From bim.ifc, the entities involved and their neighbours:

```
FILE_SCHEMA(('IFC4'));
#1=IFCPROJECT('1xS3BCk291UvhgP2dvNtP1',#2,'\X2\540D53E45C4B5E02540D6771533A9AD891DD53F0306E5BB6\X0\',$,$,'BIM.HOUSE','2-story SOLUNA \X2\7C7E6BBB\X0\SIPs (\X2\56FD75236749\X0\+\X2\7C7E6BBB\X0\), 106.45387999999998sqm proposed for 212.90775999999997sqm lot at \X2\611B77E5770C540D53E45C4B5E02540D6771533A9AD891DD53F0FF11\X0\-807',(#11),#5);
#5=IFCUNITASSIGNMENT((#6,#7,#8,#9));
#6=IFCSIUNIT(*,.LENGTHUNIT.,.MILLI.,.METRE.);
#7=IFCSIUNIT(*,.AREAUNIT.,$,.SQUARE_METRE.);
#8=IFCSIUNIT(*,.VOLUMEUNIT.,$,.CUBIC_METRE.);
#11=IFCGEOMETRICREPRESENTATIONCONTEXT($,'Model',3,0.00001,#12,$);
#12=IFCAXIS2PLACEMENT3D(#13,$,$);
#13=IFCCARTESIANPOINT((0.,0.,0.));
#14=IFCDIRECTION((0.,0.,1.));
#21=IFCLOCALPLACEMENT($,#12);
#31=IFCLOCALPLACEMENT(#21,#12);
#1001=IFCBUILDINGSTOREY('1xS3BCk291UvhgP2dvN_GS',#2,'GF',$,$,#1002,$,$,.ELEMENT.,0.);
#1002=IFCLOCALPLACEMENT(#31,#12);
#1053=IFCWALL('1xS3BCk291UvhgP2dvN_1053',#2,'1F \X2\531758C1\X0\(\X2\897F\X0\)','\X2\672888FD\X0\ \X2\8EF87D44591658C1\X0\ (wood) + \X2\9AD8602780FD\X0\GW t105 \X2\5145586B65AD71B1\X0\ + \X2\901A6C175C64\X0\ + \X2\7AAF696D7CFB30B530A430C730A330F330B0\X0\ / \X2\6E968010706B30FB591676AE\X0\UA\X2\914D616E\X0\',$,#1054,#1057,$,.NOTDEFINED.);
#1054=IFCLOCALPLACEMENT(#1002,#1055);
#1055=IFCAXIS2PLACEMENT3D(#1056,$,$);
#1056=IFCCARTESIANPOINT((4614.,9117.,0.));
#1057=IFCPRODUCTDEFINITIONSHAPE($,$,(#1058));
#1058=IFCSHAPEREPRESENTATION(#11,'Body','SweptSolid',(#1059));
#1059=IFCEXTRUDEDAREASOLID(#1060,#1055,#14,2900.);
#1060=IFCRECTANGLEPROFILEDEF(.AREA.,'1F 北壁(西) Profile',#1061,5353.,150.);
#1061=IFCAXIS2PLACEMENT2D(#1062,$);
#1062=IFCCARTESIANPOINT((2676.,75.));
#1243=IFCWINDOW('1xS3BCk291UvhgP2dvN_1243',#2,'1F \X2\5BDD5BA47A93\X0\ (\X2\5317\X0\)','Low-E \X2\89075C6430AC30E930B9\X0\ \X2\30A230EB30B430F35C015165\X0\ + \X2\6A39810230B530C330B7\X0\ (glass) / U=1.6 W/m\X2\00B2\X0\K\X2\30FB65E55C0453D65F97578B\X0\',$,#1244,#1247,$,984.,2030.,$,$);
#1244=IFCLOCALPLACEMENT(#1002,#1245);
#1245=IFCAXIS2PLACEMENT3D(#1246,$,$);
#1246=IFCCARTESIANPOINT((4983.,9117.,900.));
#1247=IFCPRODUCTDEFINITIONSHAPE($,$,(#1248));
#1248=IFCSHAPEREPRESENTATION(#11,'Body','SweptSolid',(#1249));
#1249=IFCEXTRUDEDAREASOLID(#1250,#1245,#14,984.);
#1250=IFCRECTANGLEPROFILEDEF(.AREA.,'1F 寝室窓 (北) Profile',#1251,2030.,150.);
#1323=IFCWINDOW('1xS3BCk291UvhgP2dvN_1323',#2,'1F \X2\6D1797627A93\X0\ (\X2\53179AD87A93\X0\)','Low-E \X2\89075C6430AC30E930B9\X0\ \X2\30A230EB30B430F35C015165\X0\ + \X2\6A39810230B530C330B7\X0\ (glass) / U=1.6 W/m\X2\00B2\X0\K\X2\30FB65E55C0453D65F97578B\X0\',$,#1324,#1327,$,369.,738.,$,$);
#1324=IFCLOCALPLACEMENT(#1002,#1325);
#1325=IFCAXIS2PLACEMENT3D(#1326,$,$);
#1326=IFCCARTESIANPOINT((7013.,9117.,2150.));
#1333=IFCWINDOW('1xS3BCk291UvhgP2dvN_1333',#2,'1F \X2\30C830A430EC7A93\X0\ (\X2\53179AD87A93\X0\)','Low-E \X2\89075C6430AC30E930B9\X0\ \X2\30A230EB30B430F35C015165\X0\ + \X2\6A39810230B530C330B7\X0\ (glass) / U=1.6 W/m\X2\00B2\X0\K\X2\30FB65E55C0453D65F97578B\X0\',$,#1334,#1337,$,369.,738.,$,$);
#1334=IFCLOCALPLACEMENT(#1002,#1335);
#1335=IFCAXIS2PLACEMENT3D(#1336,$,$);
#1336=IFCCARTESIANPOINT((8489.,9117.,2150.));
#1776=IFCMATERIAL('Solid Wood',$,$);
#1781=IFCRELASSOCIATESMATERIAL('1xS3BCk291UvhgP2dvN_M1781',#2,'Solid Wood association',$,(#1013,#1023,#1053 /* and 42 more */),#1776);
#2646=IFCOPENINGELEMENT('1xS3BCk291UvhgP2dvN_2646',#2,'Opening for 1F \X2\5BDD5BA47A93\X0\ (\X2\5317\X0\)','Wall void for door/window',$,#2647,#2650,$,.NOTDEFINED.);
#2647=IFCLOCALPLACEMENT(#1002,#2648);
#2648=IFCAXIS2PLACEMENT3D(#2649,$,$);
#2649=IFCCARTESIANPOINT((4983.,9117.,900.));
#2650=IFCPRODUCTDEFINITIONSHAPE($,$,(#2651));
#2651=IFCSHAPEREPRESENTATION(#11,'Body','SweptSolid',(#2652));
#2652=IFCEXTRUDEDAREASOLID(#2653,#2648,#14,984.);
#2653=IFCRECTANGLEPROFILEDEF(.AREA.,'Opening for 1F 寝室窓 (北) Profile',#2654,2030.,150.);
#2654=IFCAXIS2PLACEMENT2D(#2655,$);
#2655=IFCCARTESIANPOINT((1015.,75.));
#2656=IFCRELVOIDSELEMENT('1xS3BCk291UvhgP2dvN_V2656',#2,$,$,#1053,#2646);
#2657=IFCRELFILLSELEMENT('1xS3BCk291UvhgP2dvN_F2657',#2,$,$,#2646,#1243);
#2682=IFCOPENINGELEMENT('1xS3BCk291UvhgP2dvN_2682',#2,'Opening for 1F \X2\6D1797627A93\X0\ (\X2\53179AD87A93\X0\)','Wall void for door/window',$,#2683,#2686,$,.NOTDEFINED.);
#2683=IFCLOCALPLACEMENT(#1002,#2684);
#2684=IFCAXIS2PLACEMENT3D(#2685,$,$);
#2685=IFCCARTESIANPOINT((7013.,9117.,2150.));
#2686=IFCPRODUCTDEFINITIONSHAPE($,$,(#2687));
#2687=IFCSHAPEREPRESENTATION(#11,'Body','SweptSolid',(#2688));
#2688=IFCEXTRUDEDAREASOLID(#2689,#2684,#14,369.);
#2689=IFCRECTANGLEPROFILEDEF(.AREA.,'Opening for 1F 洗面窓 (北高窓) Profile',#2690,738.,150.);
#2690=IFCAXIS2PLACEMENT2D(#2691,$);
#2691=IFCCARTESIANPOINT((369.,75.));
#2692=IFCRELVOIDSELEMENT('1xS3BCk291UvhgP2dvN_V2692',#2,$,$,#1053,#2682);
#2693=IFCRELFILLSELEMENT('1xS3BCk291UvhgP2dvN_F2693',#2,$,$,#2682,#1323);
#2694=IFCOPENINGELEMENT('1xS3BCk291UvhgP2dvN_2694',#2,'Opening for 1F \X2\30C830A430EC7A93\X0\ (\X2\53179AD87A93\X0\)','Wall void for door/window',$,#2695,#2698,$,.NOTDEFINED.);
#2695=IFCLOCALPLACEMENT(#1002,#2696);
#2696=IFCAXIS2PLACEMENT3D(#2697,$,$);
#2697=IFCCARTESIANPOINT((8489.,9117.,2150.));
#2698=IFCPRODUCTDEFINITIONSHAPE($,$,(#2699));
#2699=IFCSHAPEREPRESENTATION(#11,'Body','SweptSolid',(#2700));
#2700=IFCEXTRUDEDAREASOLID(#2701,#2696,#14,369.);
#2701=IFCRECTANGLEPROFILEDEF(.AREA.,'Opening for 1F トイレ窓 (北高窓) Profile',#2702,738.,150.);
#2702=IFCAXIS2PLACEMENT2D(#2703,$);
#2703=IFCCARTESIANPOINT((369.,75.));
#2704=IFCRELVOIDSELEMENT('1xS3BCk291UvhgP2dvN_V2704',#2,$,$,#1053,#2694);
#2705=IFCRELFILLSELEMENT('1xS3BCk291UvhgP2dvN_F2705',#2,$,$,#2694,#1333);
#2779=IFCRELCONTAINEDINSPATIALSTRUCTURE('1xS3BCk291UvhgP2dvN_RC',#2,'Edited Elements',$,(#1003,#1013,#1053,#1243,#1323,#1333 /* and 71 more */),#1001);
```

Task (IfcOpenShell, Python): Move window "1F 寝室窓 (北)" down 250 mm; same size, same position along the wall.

```python
import numpy as np
import ifcopenshell
import ifcopenshell.api.geometry
import ifcopenshell.util.placement
import ifcopenshell.util.unit

model = ifcopenshell.open("bim.ifc")
unit_scale = ifcopenshell.util.unit.calculate_unit_scale(model)

window = model.by_id(1243)
opening = window.FillsVoids[0].RelatingOpeningElement
dz = -250.0

shift = np.array([0.0, 0.0, dz])
# The window is not placed relative to its opening, so move both.
for product in (opening, window):
    matrix = ifcopenshell.util.placement.get_local_placement(product.ObjectPlacement)
    matrix[:3, 3] += shift
    ifcopenshell.api.geometry.edit_object_placement(model, product=product, matrix=matrix, is_si=False)

print(f"moved by {dz * unit_scale:+.3f} m")

model.write("bim-out.ifc")
```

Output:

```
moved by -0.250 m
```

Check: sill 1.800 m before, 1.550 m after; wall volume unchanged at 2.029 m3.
